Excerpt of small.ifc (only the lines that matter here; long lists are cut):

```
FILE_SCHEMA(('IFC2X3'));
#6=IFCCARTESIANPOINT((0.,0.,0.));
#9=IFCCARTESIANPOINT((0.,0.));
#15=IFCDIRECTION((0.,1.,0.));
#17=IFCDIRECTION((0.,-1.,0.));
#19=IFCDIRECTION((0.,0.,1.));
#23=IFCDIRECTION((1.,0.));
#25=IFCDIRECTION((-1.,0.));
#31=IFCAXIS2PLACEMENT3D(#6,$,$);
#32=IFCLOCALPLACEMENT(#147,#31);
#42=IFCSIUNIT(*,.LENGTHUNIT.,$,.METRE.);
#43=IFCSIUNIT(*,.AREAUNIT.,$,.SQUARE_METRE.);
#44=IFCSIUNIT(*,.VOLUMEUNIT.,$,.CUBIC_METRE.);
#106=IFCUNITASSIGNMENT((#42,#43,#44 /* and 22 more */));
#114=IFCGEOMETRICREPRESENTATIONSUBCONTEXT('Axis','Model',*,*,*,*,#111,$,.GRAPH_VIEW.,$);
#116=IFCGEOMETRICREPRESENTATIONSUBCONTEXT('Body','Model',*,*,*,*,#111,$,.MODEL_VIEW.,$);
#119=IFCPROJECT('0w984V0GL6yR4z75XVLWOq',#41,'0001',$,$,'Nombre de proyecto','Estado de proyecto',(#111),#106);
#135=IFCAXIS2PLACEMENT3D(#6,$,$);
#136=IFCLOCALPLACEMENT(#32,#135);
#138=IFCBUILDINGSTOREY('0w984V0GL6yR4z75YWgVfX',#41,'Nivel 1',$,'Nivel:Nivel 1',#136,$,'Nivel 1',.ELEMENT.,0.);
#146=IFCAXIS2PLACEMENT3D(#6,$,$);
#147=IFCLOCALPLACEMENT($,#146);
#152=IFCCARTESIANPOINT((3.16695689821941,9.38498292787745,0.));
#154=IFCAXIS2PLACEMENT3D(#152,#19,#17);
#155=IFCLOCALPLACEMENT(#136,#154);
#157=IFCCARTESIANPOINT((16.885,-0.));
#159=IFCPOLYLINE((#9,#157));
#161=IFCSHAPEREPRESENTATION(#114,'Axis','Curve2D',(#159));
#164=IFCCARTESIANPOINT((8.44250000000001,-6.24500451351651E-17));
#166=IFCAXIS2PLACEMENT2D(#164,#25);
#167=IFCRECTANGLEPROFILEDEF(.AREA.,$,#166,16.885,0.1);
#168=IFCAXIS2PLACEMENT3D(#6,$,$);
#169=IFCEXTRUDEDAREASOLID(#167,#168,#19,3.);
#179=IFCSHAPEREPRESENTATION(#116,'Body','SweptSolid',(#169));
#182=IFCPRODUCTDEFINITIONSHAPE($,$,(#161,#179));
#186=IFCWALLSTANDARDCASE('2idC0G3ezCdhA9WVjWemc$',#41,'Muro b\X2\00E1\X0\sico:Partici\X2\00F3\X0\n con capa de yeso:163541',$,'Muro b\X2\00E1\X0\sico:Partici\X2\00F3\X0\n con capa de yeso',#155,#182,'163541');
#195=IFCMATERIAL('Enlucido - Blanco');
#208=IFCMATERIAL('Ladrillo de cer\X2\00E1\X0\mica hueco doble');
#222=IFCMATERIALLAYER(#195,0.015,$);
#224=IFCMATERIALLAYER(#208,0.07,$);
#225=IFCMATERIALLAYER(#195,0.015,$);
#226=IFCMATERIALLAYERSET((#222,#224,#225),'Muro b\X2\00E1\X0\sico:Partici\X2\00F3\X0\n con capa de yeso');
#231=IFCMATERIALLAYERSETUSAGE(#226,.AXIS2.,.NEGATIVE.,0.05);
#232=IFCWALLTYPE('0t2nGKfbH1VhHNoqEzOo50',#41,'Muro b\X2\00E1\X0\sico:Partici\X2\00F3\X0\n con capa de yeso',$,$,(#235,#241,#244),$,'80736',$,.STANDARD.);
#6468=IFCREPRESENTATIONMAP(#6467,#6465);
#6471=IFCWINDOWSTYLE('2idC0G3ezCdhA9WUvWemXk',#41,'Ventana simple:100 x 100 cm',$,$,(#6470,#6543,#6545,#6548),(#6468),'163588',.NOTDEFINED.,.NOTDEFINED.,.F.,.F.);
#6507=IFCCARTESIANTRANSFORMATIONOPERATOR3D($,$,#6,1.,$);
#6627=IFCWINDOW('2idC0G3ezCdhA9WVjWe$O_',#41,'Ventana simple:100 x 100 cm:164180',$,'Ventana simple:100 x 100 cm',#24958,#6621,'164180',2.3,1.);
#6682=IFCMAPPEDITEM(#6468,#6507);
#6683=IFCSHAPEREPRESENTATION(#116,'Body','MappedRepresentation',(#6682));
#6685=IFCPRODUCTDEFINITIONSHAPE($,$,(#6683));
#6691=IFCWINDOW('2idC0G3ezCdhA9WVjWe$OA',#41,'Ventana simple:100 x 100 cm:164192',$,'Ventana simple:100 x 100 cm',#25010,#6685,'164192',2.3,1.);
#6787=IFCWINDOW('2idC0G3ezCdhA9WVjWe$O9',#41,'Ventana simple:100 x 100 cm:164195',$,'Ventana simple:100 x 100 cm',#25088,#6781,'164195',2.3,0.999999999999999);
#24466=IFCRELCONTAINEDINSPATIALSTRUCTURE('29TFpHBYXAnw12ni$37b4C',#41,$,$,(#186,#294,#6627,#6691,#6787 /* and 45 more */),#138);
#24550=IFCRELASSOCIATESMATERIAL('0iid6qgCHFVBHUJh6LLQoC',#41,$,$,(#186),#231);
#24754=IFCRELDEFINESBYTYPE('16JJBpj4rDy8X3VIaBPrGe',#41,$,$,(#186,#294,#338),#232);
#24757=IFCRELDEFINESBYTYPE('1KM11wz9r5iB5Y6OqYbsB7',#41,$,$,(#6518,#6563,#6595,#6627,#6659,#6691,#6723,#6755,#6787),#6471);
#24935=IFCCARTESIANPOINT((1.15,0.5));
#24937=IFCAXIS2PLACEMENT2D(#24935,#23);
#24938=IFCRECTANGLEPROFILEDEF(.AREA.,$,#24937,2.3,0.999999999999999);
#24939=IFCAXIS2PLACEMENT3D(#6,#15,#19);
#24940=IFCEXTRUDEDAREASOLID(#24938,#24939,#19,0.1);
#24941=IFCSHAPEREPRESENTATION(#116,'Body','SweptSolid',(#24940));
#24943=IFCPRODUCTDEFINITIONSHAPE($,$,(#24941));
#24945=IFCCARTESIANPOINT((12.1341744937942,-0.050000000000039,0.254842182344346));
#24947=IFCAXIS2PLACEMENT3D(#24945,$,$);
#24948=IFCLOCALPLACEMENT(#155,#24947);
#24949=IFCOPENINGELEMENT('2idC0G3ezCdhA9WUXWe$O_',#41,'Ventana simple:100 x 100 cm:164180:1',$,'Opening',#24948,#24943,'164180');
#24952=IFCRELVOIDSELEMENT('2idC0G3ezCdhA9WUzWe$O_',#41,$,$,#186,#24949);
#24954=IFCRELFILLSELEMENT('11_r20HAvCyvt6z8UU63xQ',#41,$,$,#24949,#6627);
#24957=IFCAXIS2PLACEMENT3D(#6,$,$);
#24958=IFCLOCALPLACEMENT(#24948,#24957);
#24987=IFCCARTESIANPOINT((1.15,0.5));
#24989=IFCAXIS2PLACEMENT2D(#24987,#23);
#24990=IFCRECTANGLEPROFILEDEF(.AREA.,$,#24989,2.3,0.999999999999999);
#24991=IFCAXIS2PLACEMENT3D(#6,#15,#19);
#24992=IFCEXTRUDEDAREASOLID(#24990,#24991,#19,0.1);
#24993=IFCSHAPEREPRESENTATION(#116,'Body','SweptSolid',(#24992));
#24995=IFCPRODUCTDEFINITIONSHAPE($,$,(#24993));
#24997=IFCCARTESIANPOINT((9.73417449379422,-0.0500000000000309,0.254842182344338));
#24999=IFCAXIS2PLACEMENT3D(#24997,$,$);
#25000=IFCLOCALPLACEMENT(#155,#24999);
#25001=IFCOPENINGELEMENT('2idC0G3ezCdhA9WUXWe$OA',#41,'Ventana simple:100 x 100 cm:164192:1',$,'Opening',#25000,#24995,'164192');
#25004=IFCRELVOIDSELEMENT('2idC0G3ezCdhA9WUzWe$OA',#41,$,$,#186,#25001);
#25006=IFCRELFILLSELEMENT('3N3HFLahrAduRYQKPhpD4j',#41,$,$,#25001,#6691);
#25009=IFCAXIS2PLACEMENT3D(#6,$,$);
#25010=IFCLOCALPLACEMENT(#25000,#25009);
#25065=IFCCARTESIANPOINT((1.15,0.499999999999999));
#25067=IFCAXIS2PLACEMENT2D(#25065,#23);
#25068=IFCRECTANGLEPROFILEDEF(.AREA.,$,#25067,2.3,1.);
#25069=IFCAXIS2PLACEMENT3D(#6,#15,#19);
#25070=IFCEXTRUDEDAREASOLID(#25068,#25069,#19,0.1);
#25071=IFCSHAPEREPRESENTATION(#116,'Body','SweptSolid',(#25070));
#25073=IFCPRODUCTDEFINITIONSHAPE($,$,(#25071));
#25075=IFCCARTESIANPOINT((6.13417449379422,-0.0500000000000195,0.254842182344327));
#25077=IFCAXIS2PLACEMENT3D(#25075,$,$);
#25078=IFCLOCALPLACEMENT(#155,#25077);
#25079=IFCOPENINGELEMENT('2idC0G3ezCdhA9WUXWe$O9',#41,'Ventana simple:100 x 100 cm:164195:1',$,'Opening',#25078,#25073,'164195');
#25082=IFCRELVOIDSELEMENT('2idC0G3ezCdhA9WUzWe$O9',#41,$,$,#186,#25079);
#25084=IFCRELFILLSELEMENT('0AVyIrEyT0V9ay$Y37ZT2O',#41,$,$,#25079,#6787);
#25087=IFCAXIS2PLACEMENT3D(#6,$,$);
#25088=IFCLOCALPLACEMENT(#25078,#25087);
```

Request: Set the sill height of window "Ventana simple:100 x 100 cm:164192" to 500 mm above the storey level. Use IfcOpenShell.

```python
import numpy as np
import ifcopenshell
import ifcopenshell.api.geometry
import ifcopenshell.geom
import ifcopenshell.util.element
import ifcopenshell.util.placement
import ifcopenshell.util.shape
import ifcopenshell.util.unit

model = ifcopenshell.open("small.ifc")
unit_scale = ifcopenshell.util.unit.calculate_unit_scale(model)

window = model.by_guid("2idC0G3ezCdhA9WVjWe$OA")
opening = window.FillsVoids[0].RelatingOpeningElement
storey = ifcopenshell.util.element.get_container(window, ifc_class="IfcBuildingStorey")
level = ifcopenshell.util.placement.get_local_placement(storey.ObjectPlacement)[2, 3]

# The opening's origin need not be at the sill, so measure its lowest point.
shape = ifcopenshell.geom.create_shape(ifcopenshell.geom.settings(), opening)
bottom = ifcopenshell.util.shape.get_shape_bottom_elevation(shape, shape.geometry) / unit_scale
dz = level + 0.5 / unit_scale - bottom

shift = np.array([0.0, 0.0, dz])
# The window is placed relative to its opening, so it follows when the opening moves.
matrix = ifcopenshell.util.placement.get_local_placement(opening.ObjectPlacement)
matrix[:3, 3] += shift
ifcopenshell.api.geometry.edit_object_placement(
    model, product=opening, matrix=matrix, is_si=False, should_transform_children=True
)

print(f"moved by {dz * unit_scale:+.3f} m")

model.write("small_v2.ifc")
```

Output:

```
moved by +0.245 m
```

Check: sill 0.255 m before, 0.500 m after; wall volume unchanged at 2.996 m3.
